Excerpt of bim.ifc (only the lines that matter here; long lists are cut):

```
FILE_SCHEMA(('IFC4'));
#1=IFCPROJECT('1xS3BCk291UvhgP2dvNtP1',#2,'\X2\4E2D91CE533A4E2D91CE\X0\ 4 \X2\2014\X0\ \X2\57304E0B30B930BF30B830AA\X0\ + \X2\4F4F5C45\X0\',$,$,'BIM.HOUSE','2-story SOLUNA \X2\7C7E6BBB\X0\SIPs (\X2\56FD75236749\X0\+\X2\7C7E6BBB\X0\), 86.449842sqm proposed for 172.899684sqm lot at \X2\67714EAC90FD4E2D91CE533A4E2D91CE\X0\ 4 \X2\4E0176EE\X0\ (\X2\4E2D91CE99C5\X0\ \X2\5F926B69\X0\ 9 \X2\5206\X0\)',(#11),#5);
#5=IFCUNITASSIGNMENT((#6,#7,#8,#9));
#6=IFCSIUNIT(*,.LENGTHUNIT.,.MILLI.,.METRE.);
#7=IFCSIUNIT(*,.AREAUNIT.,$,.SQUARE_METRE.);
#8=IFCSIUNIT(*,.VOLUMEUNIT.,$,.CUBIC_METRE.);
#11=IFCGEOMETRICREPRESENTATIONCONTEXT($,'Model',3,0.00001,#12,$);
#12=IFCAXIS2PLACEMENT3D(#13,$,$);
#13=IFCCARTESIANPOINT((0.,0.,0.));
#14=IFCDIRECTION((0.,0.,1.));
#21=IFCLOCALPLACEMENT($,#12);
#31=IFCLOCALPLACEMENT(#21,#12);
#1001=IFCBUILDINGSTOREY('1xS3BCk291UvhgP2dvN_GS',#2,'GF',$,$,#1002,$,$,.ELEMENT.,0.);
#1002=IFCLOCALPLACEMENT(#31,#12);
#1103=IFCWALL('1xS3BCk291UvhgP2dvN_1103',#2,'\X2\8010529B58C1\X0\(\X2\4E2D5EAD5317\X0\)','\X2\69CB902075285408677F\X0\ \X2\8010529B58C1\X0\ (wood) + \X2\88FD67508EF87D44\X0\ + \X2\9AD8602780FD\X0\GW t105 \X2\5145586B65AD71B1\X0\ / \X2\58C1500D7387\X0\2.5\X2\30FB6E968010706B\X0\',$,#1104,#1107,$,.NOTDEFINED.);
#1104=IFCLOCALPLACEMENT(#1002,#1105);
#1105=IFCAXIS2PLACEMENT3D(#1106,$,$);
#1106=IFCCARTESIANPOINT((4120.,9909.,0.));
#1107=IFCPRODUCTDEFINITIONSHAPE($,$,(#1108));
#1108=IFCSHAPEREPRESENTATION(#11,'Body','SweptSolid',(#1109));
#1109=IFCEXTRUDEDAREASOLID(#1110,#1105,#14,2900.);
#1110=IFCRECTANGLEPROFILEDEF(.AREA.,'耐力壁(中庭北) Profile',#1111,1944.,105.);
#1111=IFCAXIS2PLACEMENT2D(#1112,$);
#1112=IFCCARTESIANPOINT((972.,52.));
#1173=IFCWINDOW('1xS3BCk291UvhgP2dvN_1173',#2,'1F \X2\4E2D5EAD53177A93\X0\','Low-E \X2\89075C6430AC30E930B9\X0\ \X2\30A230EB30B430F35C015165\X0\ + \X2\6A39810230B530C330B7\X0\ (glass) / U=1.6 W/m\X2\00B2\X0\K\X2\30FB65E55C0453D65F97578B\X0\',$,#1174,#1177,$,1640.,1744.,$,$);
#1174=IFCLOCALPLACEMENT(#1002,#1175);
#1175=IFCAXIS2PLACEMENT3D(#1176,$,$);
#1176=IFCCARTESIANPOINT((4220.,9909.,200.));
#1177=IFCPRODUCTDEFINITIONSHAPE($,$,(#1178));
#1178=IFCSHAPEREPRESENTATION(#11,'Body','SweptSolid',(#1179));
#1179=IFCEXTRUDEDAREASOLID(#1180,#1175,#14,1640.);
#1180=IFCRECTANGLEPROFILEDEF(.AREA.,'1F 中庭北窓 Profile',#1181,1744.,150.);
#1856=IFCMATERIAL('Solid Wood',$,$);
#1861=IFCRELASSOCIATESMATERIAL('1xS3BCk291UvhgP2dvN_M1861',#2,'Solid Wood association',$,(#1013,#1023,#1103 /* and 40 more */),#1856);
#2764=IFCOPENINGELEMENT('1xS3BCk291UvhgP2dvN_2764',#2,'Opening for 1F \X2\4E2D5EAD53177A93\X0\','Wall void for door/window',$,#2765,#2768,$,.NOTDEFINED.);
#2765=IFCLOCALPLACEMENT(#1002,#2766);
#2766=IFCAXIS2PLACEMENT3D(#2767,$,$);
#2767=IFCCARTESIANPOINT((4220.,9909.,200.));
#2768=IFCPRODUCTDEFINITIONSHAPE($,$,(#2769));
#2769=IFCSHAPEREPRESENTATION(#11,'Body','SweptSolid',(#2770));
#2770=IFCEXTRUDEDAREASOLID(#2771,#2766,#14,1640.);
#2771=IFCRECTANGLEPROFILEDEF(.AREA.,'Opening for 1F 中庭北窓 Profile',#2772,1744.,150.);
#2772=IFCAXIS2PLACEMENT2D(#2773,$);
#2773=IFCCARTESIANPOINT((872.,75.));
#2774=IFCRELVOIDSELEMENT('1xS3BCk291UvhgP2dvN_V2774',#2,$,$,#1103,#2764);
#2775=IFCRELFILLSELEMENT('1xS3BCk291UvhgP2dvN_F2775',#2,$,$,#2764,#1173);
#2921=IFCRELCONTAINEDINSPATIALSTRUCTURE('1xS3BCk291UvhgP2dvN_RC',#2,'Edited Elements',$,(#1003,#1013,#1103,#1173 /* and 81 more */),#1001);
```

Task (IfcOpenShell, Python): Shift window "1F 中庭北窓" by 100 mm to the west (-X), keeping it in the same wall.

```python
import ifcopenshell
import ifcopenshell.api.geometry
import ifcopenshell.util.placement
import ifcopenshell.util.unit

model = ifcopenshell.open("bim.ifc")
unit_scale = ifcopenshell.util.unit.calculate_unit_scale(model)

window = model.by_id(1173)
opening = window.FillsVoids[0].RelatingOpeningElement
wall = opening.VoidsElements[0].RelatingBuildingElement

wall_matrix = ifcopenshell.util.placement.get_local_placement(wall.ObjectPlacement)
shift = wall_matrix[:3, 0] * -0.1 / unit_scale
before = ifcopenshell.util.placement.get_local_placement(window.ObjectPlacement)[:3, 3].copy()

# The window is not placed relative to its opening, so move both.
for product in (opening, window):
    matrix = ifcopenshell.util.placement.get_local_placement(product.ObjectPlacement)
    matrix[:3, 3] += shift
    ifcopenshell.api.geometry.edit_object_placement(model, product=product, matrix=matrix, is_si=False)

after = ifcopenshell.util.placement.get_local_placement(window.ObjectPlacement)[:3, 3]
print("window moved by", (after - before).round(3) + 0.0)

model.write("bim_v2.ifc")
```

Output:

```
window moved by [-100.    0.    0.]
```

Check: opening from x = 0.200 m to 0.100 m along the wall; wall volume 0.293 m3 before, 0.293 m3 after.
